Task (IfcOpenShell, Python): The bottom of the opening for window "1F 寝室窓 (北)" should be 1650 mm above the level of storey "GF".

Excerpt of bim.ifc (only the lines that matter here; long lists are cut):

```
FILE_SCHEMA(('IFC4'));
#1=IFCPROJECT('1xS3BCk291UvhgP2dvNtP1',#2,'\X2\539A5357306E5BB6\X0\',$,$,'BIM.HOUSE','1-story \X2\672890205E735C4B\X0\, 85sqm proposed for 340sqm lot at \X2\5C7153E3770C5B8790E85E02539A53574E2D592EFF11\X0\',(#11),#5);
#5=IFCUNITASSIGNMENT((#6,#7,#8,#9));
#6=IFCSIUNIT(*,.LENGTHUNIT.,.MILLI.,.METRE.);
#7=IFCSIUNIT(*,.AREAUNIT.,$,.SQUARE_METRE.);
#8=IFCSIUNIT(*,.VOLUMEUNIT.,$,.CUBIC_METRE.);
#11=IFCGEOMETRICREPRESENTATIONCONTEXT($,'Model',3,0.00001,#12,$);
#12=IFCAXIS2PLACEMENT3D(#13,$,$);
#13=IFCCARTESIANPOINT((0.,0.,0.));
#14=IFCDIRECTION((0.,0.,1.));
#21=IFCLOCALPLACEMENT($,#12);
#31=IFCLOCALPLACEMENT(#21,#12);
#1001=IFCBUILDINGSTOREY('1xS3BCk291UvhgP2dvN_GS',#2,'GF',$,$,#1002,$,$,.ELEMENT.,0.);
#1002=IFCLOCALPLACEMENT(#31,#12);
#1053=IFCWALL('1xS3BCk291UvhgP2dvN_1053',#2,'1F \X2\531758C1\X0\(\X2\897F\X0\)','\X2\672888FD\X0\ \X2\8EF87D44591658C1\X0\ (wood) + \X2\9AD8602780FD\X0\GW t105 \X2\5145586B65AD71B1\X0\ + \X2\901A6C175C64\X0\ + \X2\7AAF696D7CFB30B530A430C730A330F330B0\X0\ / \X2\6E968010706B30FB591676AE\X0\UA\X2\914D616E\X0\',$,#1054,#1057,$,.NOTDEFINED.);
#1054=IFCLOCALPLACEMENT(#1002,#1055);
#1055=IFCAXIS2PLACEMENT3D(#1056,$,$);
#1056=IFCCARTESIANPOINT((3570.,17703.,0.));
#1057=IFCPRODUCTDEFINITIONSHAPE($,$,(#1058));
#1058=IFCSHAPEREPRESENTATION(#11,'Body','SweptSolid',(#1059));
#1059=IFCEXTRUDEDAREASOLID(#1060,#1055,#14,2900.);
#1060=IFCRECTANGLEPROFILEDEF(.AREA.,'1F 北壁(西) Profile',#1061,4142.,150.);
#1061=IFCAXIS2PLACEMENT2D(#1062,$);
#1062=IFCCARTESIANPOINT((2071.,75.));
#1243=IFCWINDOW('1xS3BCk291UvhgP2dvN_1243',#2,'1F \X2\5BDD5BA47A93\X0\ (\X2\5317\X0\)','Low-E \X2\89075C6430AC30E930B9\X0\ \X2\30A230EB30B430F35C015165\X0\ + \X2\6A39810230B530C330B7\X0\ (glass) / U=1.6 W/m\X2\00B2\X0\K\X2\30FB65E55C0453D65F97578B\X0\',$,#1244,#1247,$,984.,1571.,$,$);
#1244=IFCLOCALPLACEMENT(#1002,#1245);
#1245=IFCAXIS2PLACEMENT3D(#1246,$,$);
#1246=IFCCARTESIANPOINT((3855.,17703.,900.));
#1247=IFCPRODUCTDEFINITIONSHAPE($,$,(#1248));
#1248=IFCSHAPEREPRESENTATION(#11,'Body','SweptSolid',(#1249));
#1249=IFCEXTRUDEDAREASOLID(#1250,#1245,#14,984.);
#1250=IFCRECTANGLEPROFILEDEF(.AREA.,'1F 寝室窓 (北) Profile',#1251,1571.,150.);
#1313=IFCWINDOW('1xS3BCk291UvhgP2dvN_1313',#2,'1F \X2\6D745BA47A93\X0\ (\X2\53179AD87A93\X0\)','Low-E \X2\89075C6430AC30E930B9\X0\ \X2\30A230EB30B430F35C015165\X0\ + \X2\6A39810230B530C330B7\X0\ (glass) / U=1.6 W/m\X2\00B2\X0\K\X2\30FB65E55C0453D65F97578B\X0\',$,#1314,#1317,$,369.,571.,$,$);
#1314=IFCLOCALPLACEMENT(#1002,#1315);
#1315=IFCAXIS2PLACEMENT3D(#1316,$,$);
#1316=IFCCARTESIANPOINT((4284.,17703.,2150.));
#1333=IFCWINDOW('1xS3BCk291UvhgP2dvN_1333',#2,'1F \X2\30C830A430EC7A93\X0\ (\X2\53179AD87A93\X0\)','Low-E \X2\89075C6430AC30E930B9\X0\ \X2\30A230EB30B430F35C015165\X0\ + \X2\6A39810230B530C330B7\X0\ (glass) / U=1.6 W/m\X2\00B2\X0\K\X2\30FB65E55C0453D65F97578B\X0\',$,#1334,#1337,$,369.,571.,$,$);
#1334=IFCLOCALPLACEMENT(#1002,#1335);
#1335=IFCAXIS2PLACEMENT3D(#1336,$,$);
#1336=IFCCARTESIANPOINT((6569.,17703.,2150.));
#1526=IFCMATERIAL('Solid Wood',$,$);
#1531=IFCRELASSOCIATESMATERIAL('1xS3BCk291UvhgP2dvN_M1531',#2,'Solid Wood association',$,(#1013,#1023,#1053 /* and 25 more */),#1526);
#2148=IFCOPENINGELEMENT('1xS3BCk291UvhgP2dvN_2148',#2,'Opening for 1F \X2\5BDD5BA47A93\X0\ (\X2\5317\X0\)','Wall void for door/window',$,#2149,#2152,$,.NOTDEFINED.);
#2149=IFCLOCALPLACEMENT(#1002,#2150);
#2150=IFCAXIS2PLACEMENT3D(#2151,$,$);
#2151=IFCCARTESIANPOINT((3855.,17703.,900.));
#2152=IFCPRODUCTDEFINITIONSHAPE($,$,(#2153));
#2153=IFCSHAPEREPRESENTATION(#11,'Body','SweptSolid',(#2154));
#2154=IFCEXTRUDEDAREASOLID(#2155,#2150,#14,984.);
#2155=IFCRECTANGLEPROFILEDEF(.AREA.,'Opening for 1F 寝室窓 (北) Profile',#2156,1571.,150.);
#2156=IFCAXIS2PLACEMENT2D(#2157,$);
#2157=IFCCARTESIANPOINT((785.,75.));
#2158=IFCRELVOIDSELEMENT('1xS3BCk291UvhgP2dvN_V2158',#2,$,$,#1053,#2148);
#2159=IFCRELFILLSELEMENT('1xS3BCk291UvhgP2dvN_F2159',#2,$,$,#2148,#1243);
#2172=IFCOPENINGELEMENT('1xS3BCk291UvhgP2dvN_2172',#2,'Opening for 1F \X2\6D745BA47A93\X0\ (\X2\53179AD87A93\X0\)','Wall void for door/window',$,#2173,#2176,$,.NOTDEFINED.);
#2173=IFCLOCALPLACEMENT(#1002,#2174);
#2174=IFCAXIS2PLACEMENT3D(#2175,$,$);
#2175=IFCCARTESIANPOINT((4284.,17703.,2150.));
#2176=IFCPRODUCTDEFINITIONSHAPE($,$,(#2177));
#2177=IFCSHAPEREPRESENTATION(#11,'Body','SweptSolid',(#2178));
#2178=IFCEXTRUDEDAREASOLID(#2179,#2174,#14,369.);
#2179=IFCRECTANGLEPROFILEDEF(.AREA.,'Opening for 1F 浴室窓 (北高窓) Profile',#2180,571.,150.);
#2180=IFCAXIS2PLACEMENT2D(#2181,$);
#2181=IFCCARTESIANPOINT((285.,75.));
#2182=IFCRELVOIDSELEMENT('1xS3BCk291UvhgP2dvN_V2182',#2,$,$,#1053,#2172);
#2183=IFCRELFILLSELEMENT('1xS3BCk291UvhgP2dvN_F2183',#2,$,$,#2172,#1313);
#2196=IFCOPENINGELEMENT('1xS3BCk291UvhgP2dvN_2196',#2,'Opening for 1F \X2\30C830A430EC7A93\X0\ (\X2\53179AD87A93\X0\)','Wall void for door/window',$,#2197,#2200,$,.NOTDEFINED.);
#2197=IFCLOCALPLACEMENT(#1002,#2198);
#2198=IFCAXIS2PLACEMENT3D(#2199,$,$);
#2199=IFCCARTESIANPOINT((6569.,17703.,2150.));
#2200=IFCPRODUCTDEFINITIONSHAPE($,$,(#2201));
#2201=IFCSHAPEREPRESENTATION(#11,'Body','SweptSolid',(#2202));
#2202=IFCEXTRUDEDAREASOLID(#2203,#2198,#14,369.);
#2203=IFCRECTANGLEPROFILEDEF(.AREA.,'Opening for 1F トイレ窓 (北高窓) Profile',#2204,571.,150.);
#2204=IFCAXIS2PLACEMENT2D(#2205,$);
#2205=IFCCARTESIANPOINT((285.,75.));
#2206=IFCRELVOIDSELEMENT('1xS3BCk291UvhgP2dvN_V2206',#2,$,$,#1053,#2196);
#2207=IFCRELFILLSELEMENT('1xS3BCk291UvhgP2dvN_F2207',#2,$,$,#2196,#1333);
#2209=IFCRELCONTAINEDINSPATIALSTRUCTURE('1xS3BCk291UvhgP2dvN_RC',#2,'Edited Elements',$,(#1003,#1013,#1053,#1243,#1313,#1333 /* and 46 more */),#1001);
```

```python
import numpy as np
import ifcopenshell
import ifcopenshell.api.geometry
import ifcopenshell.geom
import ifcopenshell.util.element
import ifcopenshell.util.placement
import ifcopenshell.util.shape
import ifcopenshell.util.unit

model = ifcopenshell.open("bim.ifc")
unit_scale = ifcopenshell.util.unit.calculate_unit_scale(model)

window = model.by_guid("1xS3BCk291UvhgP2dvN_1243")
opening = window.FillsVoids[0].RelatingOpeningElement
storey = ifcopenshell.util.element.get_container(window, ifc_class="IfcBuildingStorey")
level = ifcopenshell.util.placement.get_local_placement(storey.ObjectPlacement)[2, 3]

# The opening's origin need not be at the sill, so measure its lowest point.
shape = ifcopenshell.geom.create_shape(ifcopenshell.geom.settings(), opening)
bottom = ifcopenshell.util.shape.get_shape_bottom_elevation(shape, shape.geometry) / unit_scale
dz = level + 1.65 / unit_scale - bottom

shift = np.array([0.0, 0.0, dz])
# The window is not placed relative to its opening, so move both.
for product in (opening, window):
    matrix = ifcopenshell.util.placement.get_local_placement(product.ObjectPlacement)
    matrix[:3, 3] += shift
    ifcopenshell.api.geometry.edit_object_placement(model, product=product, matrix=matrix, is_si=False)

print(f"moved by {dz * unit_scale:+.3f} m")

model.write("bim_updated.ifc")
```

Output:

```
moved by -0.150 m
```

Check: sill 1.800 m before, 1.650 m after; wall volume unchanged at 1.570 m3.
